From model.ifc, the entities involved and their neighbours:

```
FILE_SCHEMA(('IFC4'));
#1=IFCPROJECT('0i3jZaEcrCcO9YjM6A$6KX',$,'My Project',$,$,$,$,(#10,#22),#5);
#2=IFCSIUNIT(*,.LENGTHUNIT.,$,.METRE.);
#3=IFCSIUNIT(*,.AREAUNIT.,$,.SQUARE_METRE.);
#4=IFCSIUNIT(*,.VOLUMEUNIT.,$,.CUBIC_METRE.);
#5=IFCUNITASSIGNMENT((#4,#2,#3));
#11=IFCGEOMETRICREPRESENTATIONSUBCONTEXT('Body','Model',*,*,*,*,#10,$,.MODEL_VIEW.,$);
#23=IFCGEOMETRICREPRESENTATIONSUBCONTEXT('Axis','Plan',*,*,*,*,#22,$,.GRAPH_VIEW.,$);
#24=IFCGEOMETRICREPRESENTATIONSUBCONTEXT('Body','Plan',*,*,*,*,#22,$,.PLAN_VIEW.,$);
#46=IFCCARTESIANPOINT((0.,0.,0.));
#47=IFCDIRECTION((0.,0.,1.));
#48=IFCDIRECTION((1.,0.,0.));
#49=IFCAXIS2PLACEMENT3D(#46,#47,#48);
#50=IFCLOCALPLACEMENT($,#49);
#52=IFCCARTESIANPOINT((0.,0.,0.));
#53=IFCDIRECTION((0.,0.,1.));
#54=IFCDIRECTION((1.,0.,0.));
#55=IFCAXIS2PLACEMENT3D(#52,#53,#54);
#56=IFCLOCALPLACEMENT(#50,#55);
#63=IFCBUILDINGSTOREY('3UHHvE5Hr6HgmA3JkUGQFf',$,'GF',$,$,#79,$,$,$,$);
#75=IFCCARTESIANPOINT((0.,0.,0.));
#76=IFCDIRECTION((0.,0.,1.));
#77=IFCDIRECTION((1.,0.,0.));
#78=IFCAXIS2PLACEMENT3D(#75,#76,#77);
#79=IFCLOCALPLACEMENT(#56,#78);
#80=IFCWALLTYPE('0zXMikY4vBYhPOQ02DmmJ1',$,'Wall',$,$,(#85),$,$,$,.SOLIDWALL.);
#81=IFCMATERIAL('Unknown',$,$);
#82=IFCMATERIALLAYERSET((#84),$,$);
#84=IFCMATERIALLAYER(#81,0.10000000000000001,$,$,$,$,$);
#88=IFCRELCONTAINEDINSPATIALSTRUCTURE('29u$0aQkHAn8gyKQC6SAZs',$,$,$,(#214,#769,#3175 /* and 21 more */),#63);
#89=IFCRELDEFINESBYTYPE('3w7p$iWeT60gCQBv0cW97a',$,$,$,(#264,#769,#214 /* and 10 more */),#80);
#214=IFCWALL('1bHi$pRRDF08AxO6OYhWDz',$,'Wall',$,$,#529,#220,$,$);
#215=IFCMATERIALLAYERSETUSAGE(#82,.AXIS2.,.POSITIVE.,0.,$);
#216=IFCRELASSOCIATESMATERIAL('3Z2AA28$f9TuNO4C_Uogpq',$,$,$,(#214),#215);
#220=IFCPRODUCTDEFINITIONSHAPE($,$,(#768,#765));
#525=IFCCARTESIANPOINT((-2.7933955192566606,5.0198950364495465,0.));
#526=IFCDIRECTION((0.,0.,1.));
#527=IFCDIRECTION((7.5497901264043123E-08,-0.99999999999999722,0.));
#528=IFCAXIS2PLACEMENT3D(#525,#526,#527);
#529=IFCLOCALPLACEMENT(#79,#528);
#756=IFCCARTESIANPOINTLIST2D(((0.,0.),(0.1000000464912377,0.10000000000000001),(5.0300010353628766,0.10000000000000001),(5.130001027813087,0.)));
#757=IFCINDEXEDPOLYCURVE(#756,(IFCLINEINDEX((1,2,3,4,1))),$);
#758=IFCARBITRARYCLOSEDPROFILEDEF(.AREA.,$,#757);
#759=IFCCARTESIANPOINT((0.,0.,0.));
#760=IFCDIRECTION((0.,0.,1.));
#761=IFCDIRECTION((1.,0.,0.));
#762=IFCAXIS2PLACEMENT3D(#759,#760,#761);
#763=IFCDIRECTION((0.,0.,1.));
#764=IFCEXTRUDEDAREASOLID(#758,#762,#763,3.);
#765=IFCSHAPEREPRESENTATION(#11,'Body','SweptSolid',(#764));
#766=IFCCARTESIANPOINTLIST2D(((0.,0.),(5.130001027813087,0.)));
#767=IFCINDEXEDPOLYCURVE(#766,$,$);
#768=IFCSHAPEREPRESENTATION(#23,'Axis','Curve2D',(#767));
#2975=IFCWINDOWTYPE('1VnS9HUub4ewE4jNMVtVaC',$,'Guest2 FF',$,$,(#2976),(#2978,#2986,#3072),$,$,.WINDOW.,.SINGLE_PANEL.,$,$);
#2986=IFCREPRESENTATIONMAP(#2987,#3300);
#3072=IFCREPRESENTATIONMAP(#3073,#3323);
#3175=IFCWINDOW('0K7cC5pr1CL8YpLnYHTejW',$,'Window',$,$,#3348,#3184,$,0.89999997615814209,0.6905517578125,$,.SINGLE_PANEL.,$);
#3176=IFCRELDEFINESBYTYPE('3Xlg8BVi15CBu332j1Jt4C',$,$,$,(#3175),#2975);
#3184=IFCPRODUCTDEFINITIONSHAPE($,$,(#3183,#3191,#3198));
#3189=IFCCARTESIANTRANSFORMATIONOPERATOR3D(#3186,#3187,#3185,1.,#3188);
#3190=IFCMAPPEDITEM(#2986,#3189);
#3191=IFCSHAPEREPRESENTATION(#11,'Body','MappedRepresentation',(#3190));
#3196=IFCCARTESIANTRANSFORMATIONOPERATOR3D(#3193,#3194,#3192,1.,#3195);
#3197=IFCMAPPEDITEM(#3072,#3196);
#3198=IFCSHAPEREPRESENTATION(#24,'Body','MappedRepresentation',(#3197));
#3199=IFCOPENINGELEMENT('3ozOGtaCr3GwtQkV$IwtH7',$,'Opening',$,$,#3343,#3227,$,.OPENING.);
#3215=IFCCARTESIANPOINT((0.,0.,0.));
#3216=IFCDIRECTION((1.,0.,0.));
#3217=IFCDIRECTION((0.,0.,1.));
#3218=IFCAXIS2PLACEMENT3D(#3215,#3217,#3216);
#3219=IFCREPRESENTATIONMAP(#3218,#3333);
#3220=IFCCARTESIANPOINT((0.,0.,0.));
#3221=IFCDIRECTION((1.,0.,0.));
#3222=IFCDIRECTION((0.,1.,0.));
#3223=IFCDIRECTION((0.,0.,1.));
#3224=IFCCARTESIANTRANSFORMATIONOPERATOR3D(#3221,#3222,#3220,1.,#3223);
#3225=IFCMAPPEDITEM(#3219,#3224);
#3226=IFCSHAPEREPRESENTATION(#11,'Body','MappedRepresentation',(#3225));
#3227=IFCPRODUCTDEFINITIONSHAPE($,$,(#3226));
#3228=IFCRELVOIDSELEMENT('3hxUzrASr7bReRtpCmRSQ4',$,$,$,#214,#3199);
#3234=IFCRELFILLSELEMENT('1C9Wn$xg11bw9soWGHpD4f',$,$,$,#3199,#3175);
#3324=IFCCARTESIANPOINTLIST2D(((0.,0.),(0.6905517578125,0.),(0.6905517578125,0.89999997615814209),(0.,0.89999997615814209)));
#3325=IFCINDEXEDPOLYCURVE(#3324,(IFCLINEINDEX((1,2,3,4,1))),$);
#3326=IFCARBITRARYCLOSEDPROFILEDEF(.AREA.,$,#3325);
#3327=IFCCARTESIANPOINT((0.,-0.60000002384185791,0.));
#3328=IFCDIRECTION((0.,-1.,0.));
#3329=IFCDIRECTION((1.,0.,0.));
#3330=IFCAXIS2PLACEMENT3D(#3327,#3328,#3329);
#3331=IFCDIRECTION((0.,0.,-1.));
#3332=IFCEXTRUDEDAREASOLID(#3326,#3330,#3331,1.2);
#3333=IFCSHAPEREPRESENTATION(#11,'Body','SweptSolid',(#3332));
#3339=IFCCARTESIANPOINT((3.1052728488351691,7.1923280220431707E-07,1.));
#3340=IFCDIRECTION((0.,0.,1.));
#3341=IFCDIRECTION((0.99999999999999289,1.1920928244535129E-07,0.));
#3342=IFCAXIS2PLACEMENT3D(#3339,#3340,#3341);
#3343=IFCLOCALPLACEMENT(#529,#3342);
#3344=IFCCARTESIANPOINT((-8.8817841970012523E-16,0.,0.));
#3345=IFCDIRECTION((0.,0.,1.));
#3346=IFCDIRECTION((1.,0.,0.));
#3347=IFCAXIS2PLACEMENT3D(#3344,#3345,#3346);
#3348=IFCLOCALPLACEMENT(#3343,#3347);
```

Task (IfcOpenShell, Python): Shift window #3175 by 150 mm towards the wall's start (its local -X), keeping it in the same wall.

```python
import ifcopenshell
import ifcopenshell.api.geometry
import ifcopenshell.util.placement
import ifcopenshell.util.unit

model = ifcopenshell.open("model.ifc")
unit_scale = ifcopenshell.util.unit.calculate_unit_scale(model)

window = model.by_guid("0K7cC5pr1CL8YpLnYHTejW")
opening = window.FillsVoids[0].RelatingOpeningElement
wall = opening.VoidsElements[0].RelatingBuildingElement

wall_matrix = ifcopenshell.util.placement.get_local_placement(wall.ObjectPlacement)
shift = wall_matrix[:3, 0] * -0.15 / unit_scale
before = ifcopenshell.util.placement.get_local_placement(window.ObjectPlacement)[:3, 3].copy()

# The window is placed relative to its opening, so it follows when the opening moves.
matrix = ifcopenshell.util.placement.get_local_placement(opening.ObjectPlacement)
matrix[:3, 3] += shift
ifcopenshell.api.geometry.edit_object_placement(
    model, product=opening, matrix=matrix, is_si=False, should_transform_children=True
)

after = ifcopenshell.util.placement.get_local_placement(window.ObjectPlacement)[:3, 3]
print("window moved by", (after - before).round(3) + 0.0)

model.write("model_updated.ifc")
```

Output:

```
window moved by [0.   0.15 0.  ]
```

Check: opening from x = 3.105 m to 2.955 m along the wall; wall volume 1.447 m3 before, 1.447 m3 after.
